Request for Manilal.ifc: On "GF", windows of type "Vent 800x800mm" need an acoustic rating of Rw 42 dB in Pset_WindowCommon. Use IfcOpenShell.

First a look at what the model holds.

```python
import ifcopenshell
import ifcopenshell.util.element

model = ifcopenshell.open("Manilal.ifc")
print(model.schema)
storey = next(s for s in model.by_type("IfcBuildingStorey") if s.Name == "GF")
windows = [e for e in ifcopenshell.util.element.get_decomposition(storey) if e.is_a("IfcWindow")]
seen = {}
for e in windows:
    element_type = ifcopenshell.util.element.get_type(e)
    key = (element_type.Name if element_type != e and element_type else None, ifcopenshell.util.element.get_pset(e, "Pset_WindowCommon", "AcousticRating"))
    seen[key] = seen.get(key, 0) + 1
for (name, value), count in sorted(seen.items(), key=str):
    print(count, "x", name, "|", value)
```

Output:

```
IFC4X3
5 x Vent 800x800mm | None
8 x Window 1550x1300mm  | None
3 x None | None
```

```python
import ifcopenshell
import ifcopenshell.api.pset
import ifcopenshell.util.element

model = ifcopenshell.open("Manilal.ifc")

storey = next(s for s in model.by_type("IfcBuildingStorey") if s.Name == "GF")
windows = [e for e in ifcopenshell.util.element.get_decomposition(storey) if e.is_a("IfcWindow")]

count = 0
for e in windows:
    element_type = ifcopenshell.util.element.get_type(e)
    if element_type in (None, e) or element_type.Name != "Vent 800x800mm":
        continue
    # add_pset returns the element's existing set when there is one.
    pset = ifcopenshell.api.pset.add_pset(model, product=e, name="Pset_WindowCommon")
    ifcopenshell.api.pset.edit_pset(model, pset=pset, properties={"AcousticRating": "Rw 42 dB"})
    count += 1

print(count, "windows updated")

model.write("Manilal_v2.ifc")
```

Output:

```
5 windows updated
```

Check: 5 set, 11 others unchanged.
